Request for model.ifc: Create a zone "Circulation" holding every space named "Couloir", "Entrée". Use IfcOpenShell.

First a look at what the model holds.

```python
import ifcopenshell

model = ifcopenshell.open("model.ifc")
print(model.schema)
seen = {}
for space in model.by_type("IfcSpace"):
    seen[space.LongName] = seen.get(space.LongName, 0) + 1
for name, count in sorted(seen.items(), key=str):
    print(count, "x", name)
print("zones:", [z.Name for z in model.by_type("IfcZone")][:20])
```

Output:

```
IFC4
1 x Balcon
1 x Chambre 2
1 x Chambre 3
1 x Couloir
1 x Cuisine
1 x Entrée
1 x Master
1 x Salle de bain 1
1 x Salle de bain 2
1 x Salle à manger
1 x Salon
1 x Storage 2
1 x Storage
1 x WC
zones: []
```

```python
import ifcopenshell
import ifcopenshell.api.group
import ifcopenshell.api.root

model = ifcopenshell.open("model.ifc")

names = {"Couloir", "Entrée"}
spaces = [s for s in model.by_type("IfcSpace") if s.LongName in names]

zone = ifcopenshell.api.root.create_entity(model, ifc_class="IfcZone", name="Circulation")
ifcopenshell.api.group.assign_group(model, products=spaces, group=zone)
print(len(spaces), "spaces in", zone.Name)

model.write("model_updated.ifc")
```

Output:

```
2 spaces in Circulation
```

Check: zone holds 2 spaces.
